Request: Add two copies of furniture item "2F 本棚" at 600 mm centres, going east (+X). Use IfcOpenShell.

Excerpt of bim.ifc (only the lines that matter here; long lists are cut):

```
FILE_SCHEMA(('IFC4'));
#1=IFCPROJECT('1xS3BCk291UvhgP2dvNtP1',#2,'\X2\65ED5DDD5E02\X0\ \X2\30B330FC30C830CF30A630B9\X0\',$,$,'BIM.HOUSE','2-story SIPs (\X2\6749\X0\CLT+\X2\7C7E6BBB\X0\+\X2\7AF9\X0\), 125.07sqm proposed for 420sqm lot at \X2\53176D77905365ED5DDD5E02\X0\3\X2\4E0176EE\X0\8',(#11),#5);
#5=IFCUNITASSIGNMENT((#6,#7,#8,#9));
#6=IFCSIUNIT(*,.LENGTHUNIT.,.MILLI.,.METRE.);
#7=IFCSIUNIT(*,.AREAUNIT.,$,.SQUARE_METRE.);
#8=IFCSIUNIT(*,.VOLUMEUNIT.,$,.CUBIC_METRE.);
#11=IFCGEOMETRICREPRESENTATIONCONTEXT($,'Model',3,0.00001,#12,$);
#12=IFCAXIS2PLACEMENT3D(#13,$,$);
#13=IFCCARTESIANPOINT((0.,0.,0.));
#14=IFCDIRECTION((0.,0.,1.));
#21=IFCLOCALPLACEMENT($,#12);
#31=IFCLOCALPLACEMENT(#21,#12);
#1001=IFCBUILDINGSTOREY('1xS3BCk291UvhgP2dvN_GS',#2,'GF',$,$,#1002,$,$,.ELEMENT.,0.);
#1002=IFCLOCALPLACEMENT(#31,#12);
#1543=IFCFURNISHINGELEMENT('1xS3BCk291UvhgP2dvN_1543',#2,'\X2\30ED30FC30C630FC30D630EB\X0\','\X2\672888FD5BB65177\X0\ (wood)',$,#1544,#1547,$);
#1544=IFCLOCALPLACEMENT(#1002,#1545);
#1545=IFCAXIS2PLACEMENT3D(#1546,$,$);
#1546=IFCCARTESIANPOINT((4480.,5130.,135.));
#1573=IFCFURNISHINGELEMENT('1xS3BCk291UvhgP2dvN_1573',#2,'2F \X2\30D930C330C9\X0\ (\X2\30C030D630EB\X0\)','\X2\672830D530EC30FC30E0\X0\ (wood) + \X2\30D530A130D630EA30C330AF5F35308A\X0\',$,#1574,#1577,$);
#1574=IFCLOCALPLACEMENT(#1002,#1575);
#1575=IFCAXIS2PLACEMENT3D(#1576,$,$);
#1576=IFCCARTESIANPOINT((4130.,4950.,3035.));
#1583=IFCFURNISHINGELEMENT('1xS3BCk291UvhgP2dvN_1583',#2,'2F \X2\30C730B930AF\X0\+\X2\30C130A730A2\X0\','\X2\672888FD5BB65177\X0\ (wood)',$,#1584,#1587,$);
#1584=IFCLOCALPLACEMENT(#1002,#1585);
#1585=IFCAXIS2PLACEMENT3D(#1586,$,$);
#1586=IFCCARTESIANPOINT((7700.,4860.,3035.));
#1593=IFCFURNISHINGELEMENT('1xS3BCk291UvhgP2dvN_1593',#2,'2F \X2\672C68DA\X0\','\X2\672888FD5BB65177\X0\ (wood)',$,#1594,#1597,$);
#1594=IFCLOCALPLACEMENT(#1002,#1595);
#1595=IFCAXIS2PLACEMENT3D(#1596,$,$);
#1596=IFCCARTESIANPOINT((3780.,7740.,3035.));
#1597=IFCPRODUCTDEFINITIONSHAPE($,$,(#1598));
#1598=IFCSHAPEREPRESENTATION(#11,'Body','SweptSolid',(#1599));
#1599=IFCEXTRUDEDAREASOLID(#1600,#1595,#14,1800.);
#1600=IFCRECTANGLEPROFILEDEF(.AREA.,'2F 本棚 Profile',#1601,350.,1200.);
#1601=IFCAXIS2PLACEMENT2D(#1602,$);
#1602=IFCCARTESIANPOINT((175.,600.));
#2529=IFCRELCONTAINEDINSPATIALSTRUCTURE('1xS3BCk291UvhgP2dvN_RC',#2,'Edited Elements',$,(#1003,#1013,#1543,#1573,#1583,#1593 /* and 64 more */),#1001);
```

```python
import numpy as np
import ifcopenshell
import ifcopenshell.api.geometry
import ifcopenshell.api.root
import ifcopenshell.util.element
import ifcopenshell.util.placement
import ifcopenshell.util.unit

model = ifcopenshell.open("bim.ifc")
unit_scale = ifcopenshell.util.unit.calculate_unit_scale(model)


def reuse_history(source, copy):
    """copy_class also copies each property set's owner history, people and application; keep the originals."""
    for rel in copy.IsDefinedBy:
        if rel.is_a("IfcRelDefinesByProperties") and (history := rel.RelatingPropertyDefinition.OwnerHistory):
            rel.RelatingPropertyDefinition.OwnerHistory = source.OwnerHistory
            ifcopenshell.util.element.remove_deep2(model, history)


source = model.by_guid("1xS3BCk291UvhgP2dvN_1593")
base = ifcopenshell.util.placement.get_local_placement(source.ObjectPlacement)
step = np.array([1.0, 0.0, 0.0]) * 0.6 / unit_scale

for i in range(1, 3):
    copy = ifcopenshell.api.root.copy_class(model, product=source)
    copy.Representation = ifcopenshell.util.element.copy_deep(
        model, source.Representation, exclude=["IfcGeometricRepresentationContext", "IfcRepresentationMap"]
    )
    reuse_history(source, copy)
    matrix = base.copy()
    matrix[:3, 3] += i * step
    print("added at", matrix[:3, 3].round(3) + 0.0)
    ifcopenshell.api.geometry.edit_object_placement(model, product=copy, matrix=matrix, is_si=False)

model.write("bim_v2.ifc")
```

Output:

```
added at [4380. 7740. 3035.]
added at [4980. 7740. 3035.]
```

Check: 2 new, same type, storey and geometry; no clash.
